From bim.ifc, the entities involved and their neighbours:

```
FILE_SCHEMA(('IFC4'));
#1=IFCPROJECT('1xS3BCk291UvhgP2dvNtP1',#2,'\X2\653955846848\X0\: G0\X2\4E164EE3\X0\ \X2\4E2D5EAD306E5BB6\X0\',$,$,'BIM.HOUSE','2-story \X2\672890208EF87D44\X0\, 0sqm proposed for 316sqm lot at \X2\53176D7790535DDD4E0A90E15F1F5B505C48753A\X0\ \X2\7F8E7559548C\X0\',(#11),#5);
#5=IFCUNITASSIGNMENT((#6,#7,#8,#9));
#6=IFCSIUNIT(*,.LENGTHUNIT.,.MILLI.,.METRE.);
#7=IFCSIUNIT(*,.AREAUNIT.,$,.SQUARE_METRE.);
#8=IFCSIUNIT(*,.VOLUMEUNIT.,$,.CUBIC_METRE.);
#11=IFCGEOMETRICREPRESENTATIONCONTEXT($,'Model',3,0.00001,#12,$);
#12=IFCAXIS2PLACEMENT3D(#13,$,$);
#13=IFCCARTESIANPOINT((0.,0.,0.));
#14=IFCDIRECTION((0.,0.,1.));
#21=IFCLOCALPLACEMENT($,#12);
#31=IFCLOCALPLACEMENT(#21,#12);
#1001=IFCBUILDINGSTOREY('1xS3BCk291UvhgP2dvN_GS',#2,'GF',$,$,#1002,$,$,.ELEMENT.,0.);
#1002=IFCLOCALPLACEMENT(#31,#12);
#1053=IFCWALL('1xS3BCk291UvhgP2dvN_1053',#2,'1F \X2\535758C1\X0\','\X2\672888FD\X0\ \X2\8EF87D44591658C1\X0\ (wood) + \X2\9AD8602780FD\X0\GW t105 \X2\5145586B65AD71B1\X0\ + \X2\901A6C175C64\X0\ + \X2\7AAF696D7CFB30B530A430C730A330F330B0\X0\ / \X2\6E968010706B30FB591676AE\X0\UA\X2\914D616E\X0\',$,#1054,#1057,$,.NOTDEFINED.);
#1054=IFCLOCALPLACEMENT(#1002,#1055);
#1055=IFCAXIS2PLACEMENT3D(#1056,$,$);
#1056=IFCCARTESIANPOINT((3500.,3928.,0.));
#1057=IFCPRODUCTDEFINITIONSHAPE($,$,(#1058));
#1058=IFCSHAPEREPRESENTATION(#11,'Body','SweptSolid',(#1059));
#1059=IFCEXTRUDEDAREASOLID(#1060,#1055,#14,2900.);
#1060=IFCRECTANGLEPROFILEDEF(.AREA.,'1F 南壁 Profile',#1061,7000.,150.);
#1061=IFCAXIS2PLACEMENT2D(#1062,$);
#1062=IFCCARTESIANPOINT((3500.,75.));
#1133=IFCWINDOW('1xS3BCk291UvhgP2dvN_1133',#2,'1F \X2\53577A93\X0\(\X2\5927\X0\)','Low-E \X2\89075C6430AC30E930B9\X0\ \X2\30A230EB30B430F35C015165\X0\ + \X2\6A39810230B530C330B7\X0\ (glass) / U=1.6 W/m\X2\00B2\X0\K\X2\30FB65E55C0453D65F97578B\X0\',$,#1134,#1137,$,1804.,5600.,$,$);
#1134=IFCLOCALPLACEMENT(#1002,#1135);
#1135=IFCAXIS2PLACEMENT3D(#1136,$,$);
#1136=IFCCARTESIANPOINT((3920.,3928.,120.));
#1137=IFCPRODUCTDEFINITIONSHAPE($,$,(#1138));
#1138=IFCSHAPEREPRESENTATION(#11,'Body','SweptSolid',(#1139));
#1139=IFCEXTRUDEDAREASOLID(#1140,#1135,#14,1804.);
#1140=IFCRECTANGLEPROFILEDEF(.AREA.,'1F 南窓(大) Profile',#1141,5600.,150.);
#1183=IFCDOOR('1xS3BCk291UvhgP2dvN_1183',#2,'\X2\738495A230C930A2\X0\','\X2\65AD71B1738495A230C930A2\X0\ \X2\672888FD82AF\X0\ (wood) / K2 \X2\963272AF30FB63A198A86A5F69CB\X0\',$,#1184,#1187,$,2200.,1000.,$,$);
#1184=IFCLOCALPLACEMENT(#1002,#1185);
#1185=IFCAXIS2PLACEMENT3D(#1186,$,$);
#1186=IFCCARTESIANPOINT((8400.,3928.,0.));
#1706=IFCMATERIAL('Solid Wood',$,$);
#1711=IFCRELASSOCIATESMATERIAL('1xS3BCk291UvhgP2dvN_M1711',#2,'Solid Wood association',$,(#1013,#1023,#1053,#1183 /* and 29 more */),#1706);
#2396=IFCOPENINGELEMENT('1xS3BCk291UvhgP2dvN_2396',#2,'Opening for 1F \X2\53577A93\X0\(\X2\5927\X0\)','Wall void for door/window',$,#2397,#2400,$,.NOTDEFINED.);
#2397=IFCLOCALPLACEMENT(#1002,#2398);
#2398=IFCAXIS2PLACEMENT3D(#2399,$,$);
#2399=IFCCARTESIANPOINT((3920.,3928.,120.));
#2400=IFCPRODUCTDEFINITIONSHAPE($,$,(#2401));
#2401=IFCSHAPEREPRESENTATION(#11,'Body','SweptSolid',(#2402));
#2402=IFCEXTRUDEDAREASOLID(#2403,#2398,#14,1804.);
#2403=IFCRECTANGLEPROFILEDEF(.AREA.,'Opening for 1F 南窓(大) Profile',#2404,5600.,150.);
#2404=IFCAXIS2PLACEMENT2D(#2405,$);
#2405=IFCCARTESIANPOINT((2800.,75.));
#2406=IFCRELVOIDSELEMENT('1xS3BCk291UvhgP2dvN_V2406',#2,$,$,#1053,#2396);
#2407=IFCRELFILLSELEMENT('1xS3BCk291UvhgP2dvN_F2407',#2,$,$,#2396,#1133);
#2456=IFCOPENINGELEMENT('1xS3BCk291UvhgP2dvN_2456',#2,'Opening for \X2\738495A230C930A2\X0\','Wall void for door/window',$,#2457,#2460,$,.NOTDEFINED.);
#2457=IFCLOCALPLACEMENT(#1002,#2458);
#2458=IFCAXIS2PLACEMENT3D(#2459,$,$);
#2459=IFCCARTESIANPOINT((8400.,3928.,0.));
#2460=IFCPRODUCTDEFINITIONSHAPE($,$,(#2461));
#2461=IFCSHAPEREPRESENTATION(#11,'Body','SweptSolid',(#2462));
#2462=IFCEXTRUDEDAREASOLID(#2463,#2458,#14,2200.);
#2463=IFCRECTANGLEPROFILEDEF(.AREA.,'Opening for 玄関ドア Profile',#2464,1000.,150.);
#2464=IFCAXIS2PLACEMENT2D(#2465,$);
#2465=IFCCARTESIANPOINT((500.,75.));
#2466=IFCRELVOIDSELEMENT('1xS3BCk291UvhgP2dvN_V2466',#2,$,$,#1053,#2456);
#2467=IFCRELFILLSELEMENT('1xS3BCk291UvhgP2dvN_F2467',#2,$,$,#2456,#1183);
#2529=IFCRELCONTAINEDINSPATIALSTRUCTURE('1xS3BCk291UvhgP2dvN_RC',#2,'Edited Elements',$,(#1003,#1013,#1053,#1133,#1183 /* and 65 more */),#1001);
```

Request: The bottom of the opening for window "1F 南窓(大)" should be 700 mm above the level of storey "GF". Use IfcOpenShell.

```python
import numpy as np
import ifcopenshell
import ifcopenshell.api.geometry
import ifcopenshell.geom
import ifcopenshell.util.element
import ifcopenshell.util.placement
import ifcopenshell.util.shape
import ifcopenshell.util.unit

model = ifcopenshell.open("bim.ifc")
unit_scale = ifcopenshell.util.unit.calculate_unit_scale(model)

window = model.by_guid("1xS3BCk291UvhgP2dvN_1133")
opening = window.FillsVoids[0].RelatingOpeningElement
storey = ifcopenshell.util.element.get_container(window, ifc_class="IfcBuildingStorey")
level = ifcopenshell.util.placement.get_local_placement(storey.ObjectPlacement)[2, 3]

# The opening's origin need not be at the sill, so measure its lowest point.
shape = ifcopenshell.geom.create_shape(ifcopenshell.geom.settings(), opening)
bottom = ifcopenshell.util.shape.get_shape_bottom_elevation(shape, shape.geometry) / unit_scale
dz = level + 0.7 / unit_scale - bottom

shift = np.array([0.0, 0.0, dz])
# The window is not placed relative to its opening, so move both.
for product in (opening, window):
    matrix = ifcopenshell.util.placement.get_local_placement(product.ObjectPlacement)
    matrix[:3, 3] += shift
    ifcopenshell.api.geometry.edit_object_placement(model, product=product, matrix=matrix, is_si=False)

print(f"moved by {dz * unit_scale:+.3f} m")

model.write("bim_edited.ifc")
```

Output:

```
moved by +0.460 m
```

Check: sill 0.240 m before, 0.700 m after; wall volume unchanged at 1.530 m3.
